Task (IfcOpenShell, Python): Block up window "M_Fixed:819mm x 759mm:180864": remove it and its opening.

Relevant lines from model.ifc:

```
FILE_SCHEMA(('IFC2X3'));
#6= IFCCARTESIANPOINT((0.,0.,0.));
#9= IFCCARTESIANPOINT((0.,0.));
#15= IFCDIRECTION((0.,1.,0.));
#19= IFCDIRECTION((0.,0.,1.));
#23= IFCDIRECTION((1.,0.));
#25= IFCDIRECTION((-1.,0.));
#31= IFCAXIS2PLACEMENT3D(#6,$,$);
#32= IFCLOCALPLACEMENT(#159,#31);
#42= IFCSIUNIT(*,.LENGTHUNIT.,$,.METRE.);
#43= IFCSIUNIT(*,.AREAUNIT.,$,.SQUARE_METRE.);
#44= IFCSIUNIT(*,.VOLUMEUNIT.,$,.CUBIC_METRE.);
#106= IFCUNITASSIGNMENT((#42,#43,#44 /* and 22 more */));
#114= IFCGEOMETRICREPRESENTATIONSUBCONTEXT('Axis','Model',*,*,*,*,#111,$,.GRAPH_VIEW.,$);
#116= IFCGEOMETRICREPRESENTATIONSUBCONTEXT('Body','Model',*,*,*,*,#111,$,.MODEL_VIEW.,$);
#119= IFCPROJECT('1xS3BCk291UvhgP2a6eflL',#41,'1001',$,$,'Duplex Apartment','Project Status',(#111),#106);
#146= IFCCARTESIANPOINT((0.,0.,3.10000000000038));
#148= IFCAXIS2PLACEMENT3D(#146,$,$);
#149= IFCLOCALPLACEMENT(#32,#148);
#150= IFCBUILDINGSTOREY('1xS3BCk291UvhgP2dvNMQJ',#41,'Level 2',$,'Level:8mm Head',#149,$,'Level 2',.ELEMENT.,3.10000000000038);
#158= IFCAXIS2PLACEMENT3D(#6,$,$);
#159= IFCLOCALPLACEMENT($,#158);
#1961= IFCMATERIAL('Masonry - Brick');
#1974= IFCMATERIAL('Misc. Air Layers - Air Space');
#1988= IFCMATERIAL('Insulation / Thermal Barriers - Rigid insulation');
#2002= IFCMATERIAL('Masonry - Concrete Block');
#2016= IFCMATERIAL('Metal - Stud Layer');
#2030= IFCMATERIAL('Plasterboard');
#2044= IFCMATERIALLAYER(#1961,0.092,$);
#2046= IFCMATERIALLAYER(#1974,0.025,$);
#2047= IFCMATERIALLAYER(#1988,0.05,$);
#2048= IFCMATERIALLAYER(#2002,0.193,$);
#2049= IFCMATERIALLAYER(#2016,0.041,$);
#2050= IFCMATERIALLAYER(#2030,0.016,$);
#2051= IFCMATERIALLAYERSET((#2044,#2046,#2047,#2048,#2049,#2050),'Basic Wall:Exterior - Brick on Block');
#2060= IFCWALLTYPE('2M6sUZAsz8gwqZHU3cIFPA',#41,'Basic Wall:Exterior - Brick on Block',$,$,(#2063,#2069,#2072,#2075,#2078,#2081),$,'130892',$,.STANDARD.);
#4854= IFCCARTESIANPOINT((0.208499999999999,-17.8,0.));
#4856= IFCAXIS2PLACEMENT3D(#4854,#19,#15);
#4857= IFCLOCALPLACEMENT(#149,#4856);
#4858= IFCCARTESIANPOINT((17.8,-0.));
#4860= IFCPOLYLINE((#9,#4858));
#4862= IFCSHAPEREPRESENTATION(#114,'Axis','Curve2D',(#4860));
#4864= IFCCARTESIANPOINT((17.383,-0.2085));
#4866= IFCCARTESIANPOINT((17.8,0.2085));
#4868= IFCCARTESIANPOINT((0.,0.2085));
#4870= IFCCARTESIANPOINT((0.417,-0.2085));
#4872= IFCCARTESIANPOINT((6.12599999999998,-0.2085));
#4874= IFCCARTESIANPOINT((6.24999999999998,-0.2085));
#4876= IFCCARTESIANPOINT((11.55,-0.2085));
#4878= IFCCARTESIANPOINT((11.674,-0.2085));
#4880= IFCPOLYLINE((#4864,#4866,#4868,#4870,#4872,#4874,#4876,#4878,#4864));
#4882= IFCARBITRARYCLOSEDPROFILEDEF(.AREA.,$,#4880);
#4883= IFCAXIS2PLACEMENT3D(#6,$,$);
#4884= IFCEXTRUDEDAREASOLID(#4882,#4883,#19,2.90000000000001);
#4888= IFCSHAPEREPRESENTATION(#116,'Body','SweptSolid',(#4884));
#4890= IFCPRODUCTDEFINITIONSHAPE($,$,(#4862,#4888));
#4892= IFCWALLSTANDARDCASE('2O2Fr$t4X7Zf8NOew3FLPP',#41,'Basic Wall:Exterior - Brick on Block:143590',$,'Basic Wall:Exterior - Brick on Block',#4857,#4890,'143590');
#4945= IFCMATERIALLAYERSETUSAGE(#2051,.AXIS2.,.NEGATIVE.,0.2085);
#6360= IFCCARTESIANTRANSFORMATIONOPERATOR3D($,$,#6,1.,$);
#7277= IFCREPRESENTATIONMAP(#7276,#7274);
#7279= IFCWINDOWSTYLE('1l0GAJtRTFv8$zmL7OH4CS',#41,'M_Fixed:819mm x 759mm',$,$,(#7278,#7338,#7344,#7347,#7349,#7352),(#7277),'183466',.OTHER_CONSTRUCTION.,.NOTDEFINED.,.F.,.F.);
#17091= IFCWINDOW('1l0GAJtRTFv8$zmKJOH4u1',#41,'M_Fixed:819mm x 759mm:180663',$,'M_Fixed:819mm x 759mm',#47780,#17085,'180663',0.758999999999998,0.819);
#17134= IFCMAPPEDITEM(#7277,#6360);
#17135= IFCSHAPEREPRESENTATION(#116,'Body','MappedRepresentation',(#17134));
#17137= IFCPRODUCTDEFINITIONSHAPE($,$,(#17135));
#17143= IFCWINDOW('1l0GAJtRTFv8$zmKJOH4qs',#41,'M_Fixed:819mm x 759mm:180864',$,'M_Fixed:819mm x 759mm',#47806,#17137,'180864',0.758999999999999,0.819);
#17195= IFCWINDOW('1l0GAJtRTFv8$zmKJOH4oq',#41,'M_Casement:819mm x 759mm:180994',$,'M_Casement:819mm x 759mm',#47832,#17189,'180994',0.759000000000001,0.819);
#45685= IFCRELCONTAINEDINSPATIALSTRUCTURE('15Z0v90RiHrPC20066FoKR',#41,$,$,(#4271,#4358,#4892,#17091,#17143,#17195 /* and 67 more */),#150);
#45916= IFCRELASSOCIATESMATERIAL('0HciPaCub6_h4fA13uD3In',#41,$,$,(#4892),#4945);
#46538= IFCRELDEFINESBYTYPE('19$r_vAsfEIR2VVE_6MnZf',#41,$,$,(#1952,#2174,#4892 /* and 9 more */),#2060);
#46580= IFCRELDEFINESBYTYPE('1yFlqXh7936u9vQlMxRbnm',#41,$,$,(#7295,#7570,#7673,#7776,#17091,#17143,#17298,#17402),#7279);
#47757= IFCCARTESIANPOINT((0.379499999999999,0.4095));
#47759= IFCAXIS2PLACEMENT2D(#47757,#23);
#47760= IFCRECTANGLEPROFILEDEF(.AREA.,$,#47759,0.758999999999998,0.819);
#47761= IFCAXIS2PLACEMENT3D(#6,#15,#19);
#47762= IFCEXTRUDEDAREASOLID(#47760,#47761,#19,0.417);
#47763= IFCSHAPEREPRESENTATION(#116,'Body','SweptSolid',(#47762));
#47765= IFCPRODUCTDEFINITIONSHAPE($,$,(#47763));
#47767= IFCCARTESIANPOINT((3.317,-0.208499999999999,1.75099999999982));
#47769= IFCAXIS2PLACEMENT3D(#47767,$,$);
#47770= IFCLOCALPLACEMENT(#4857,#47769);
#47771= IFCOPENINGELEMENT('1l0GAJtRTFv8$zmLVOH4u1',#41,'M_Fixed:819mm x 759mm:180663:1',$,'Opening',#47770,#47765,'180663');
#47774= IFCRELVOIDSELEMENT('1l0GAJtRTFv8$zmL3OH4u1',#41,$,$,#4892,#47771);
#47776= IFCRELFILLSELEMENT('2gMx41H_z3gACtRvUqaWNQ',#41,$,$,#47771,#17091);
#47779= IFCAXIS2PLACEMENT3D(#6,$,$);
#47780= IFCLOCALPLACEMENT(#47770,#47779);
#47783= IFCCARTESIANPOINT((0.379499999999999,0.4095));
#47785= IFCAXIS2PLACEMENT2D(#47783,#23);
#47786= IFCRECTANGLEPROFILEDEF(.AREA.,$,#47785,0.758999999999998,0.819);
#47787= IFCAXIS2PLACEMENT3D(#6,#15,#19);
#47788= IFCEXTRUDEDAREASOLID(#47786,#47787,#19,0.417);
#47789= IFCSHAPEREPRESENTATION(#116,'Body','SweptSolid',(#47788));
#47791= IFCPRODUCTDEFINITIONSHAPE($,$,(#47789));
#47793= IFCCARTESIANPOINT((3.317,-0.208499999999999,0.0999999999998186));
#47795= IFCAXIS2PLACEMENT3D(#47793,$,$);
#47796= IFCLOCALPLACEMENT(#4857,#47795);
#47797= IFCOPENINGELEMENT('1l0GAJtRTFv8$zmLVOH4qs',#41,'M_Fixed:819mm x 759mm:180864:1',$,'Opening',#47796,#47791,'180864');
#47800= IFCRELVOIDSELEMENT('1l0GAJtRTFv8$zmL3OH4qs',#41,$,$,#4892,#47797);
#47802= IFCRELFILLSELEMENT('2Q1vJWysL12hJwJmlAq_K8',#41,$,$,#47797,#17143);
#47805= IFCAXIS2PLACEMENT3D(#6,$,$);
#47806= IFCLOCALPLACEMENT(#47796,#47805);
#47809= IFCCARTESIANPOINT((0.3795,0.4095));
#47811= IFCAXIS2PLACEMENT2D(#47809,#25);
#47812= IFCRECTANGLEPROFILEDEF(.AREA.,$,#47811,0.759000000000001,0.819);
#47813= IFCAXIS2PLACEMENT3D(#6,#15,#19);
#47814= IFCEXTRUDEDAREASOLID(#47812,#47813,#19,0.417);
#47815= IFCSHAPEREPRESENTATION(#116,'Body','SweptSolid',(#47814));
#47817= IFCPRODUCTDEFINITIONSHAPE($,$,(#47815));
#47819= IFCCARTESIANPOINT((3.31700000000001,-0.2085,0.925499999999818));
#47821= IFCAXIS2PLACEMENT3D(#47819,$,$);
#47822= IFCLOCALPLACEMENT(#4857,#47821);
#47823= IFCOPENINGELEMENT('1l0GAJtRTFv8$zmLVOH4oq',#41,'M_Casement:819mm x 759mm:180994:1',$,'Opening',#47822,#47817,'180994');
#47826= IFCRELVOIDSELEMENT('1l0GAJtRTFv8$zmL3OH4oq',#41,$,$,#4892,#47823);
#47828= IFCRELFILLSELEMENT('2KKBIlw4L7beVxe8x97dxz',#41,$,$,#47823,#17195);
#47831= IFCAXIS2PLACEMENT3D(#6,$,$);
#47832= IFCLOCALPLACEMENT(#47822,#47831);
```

```python
import ifcopenshell
import ifcopenshell.api.feature
import ifcopenshell.api.root
import ifcopenshell.geom
import ifcopenshell.util.shape

model = ifcopenshell.open("model.ifc")
settings = ifcopenshell.geom.settings()


def volume(element):
    """Net volume in cubic metres, openings subtracted."""
    shape = ifcopenshell.geom.create_shape(settings, element)
    return ifcopenshell.util.shape.get_volume(shape.geometry)


window = model.by_guid("1l0GAJtRTFv8$zmKJOH4qs")
opening = window.FillsVoids[0].RelatingOpeningElement
wall = opening.VoidsElements[0].RelatingBuildingElement
before = volume(wall)

ifcopenshell.api.root.remove_product(model, product=window)
ifcopenshell.api.feature.remove_feature(model, feature=opening)

after = volume(wall)

print(f"wall volume {before:.3f} -> {after:.3f} m3")

model.write("model_v2.ifc")
```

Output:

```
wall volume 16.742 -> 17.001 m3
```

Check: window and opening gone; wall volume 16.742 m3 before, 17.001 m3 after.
